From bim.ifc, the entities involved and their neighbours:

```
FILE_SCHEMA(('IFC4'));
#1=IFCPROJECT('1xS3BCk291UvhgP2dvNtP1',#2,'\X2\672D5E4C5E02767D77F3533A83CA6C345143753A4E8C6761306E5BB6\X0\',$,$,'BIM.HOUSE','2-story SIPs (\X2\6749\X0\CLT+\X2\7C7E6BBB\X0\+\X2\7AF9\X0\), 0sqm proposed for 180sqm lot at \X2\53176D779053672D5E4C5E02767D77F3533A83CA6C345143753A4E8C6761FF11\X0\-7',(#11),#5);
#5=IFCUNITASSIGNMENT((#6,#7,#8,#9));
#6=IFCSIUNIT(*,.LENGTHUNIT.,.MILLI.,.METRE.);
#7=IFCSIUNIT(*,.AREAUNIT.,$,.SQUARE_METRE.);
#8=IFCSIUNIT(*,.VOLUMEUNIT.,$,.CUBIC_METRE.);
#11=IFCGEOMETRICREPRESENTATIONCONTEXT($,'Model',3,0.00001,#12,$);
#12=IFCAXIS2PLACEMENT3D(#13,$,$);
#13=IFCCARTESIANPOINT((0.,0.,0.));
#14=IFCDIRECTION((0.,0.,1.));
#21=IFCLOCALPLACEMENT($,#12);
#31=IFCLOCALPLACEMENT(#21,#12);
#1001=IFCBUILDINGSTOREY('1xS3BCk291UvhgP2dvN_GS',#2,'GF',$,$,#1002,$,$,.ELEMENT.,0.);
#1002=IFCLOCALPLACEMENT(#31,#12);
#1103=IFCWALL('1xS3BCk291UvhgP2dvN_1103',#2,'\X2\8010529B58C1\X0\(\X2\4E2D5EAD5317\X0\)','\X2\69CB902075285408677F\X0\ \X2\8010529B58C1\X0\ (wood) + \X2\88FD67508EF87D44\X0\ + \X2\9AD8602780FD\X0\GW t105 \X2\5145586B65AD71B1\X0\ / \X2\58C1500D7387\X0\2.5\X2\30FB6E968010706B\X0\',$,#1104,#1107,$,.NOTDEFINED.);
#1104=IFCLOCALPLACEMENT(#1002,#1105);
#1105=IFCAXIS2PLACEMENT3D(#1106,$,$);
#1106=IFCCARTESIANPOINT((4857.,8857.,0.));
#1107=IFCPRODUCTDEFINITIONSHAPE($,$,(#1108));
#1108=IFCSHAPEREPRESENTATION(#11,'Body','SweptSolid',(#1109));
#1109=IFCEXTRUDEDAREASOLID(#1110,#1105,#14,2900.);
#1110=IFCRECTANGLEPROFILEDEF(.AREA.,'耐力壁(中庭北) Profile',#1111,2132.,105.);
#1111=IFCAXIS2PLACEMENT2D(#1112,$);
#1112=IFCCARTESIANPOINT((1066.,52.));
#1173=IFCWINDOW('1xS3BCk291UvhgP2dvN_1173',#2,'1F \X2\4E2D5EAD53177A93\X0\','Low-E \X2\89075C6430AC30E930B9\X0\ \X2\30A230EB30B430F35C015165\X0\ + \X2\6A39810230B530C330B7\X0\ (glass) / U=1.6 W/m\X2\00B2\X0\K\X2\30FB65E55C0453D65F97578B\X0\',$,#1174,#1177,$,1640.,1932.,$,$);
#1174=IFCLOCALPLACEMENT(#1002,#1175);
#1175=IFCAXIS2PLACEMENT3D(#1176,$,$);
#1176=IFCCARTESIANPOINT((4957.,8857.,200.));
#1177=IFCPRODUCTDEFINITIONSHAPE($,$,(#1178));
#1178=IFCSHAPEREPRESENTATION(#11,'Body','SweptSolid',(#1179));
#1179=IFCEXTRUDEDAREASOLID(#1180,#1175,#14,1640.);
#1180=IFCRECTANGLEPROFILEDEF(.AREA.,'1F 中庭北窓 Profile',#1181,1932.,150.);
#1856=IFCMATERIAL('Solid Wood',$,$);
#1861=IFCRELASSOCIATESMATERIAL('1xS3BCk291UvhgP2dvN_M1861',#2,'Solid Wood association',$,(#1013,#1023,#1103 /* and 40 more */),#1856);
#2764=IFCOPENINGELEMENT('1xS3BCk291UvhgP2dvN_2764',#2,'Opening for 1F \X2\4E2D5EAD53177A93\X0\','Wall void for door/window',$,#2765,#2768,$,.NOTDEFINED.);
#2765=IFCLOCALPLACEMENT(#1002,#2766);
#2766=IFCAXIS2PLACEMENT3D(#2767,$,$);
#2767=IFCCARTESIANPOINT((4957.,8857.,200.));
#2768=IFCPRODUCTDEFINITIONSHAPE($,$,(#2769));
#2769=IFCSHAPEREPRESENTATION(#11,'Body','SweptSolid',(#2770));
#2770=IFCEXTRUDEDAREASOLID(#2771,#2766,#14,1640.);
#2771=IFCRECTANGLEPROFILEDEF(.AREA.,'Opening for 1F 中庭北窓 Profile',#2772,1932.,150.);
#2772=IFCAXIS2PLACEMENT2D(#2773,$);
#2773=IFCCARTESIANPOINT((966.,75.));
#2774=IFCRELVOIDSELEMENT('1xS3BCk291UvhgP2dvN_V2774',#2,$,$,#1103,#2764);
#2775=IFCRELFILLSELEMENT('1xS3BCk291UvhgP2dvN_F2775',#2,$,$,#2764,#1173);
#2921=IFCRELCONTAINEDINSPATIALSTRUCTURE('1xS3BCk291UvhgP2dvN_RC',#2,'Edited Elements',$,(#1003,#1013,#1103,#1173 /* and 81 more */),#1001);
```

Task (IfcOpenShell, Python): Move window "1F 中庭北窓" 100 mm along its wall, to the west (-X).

```python
import ifcopenshell
import ifcopenshell.api.geometry
import ifcopenshell.util.placement

model = ifcopenshell.open("bim.ifc")

window = model.by_guid("1xS3BCk291UvhgP2dvN_1173")
opening = window.FillsVoids[0].RelatingOpeningElement
wall = opening.VoidsElements[0].RelatingBuildingElement

wall_matrix = ifcopenshell.util.placement.get_local_placement(wall.ObjectPlacement)
shift = wall_matrix[:3, 0] * -100.0
before = ifcopenshell.util.placement.get_local_placement(window.ObjectPlacement)[:3, 3].copy()

# The window is not placed relative to its opening, so move both.
for product in (opening, window):
    matrix = ifcopenshell.util.placement.get_local_placement(product.ObjectPlacement)
    matrix[:3, 3] += shift
    ifcopenshell.api.geometry.edit_object_placement(model, product=product, matrix=matrix, is_si=False)

after = ifcopenshell.util.placement.get_local_placement(window.ObjectPlacement)[:3, 3]
print("window moved by", (after - before).round(3) + 0.0)

model.write("bim_v2.ifc")
```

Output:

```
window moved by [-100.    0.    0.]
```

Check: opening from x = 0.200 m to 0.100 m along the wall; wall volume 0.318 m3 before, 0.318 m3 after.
